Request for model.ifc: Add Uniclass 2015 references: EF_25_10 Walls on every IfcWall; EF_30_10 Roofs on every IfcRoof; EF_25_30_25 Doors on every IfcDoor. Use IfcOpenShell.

First a look at what the model holds.

```python
import ifcopenshell

model = ifcopenshell.open("model.ifc")
print(model.schema)
print("classifications:", [c.Name for c in model.by_type("IfcClassification")])
for ifc_class in ("IfcDoor", "IfcRoof", "IfcStair", "IfcWall", "IfcWindow"):
    print(ifc_class, len(model.by_type(ifc_class)))
```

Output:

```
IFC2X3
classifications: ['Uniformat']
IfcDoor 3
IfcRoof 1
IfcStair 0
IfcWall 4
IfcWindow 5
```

```python
import ifcopenshell
import ifcopenshell.api.classification

model = ifcopenshell.open("model.ifc")

# IFC2X3 requires Source and Edition and has no link from the project to the system.
system = model.create_entity("IfcClassification", Source="NBS", Edition="2015", Name="Uniclass 2015")

codes = {
    "IfcWall": ("EF_25_10", "Walls"),
    "IfcRoof": ("EF_30_10", "Roofs"),
    "IfcDoor": ("EF_25_30_25", "Doors"),
}
for ifc_class, (code, name) in codes.items():
    products = model.by_type(ifc_class)
    ifcopenshell.api.classification.add_reference(
        model, products=products, classification=system, identification=code, name=name
    )
    print(code, len(products))

model.write("model-out.ifc")
```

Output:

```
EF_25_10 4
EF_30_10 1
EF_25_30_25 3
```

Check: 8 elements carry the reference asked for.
